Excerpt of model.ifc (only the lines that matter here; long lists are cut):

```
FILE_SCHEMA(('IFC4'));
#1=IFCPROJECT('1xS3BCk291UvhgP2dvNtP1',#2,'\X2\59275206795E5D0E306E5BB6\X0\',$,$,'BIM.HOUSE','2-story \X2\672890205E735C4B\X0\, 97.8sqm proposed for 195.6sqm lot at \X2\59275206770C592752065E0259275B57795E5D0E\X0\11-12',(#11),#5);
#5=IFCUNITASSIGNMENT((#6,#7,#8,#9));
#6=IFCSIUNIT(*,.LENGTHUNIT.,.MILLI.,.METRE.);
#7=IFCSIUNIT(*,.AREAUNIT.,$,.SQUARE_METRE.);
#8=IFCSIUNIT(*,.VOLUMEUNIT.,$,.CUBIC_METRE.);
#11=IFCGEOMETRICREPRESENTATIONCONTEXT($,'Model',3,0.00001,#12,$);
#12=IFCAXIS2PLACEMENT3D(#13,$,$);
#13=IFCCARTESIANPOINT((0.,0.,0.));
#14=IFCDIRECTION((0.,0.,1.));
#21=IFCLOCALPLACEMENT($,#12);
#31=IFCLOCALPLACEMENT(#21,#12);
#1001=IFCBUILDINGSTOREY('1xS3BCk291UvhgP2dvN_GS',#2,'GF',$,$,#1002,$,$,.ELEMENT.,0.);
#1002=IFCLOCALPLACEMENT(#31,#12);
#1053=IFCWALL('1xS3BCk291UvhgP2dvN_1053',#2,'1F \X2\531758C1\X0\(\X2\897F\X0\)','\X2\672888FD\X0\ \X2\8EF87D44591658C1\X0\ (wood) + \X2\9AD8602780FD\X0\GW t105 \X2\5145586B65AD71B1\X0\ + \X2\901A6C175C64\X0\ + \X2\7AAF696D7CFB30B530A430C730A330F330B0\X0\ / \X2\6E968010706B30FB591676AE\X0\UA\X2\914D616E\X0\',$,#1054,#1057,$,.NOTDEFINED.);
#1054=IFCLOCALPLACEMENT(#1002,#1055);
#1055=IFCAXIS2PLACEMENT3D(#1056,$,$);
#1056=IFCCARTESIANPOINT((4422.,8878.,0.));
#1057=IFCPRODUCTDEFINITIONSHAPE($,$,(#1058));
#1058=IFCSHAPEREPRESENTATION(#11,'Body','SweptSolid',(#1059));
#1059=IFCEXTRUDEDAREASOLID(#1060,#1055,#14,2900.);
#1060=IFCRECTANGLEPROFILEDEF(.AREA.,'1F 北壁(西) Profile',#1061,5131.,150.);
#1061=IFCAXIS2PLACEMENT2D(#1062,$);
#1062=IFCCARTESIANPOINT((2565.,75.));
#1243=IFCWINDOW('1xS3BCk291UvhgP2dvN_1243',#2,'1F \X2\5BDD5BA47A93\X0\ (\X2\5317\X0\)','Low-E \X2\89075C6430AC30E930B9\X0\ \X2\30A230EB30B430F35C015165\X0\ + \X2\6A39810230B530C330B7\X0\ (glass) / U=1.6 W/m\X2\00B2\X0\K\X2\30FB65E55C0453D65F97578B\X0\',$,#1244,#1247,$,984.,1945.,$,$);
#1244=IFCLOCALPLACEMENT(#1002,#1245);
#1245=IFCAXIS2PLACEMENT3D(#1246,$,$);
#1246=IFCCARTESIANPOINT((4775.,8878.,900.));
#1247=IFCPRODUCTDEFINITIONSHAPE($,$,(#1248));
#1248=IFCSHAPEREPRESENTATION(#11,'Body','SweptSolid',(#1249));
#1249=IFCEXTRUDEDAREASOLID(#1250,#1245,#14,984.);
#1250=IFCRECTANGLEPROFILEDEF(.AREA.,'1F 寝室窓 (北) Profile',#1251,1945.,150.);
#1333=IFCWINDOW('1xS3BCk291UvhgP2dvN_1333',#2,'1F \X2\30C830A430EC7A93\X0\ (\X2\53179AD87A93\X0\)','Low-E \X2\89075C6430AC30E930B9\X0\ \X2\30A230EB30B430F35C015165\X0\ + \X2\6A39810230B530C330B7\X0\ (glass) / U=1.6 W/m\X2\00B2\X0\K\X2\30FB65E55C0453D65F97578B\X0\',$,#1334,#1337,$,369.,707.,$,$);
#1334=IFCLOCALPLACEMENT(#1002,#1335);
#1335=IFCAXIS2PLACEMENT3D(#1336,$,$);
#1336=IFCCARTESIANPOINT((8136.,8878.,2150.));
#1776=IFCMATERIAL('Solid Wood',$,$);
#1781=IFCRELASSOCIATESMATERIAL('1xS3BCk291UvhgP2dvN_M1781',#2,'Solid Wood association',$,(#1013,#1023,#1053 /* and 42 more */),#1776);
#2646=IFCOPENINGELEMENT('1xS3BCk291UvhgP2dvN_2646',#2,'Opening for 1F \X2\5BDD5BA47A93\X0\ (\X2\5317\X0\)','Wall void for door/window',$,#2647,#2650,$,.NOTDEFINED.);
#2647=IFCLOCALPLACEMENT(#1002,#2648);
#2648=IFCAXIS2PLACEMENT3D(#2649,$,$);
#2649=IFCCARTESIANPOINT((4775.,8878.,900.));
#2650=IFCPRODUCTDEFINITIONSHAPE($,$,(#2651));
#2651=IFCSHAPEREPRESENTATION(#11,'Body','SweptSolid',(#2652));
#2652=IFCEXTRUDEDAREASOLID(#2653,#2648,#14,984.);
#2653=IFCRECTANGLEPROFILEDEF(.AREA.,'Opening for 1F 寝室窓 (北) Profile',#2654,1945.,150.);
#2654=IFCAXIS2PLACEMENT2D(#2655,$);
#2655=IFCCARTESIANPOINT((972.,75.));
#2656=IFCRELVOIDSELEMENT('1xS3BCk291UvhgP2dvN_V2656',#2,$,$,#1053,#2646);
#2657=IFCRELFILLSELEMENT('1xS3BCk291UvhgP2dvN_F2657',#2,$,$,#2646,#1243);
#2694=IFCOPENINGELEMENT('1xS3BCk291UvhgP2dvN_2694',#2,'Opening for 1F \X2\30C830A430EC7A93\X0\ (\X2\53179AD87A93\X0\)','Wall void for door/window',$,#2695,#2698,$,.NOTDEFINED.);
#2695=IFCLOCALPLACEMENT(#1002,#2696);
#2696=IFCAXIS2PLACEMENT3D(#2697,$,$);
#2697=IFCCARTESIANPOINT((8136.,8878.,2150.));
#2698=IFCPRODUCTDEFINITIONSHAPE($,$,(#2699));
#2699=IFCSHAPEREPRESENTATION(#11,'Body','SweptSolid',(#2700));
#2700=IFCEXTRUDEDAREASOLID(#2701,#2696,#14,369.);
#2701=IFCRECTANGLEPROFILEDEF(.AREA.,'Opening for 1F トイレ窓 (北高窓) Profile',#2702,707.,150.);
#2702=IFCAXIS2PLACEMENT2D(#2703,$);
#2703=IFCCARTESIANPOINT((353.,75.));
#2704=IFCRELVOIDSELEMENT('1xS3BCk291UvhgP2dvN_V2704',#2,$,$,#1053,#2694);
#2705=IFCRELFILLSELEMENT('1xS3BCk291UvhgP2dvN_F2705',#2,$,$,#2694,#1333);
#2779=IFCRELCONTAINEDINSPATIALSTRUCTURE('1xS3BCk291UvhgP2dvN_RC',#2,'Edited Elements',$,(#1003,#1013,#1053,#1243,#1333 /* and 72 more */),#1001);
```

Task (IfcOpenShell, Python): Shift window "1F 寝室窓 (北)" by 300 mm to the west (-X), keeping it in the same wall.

```python
import ifcopenshell
import ifcopenshell.api.geometry
import ifcopenshell.util.placement
import ifcopenshell.util.unit

model = ifcopenshell.open("model.ifc")
unit_scale = ifcopenshell.util.unit.calculate_unit_scale(model)

window = model.by_guid("1xS3BCk291UvhgP2dvN_1243")
opening = window.FillsVoids[0].RelatingOpeningElement
wall = opening.VoidsElements[0].RelatingBuildingElement

wall_matrix = ifcopenshell.util.placement.get_local_placement(wall.ObjectPlacement)
shift = wall_matrix[:3, 0] * -0.3 / unit_scale
before = ifcopenshell.util.placement.get_local_placement(window.ObjectPlacement)[:3, 3].copy()

# The window is not placed relative to its opening, so move both.
for product in (opening, window):
    matrix = ifcopenshell.util.placement.get_local_placement(product.ObjectPlacement)
    matrix[:3, 3] += shift
    ifcopenshell.api.geometry.edit_object_placement(model, product=product, matrix=matrix, is_si=False)

after = ifcopenshell.util.placement.get_local_placement(window.ObjectPlacement)[:3, 3]
print("window moved by", (after - before).round(3) + 0.0)

model.write("model_v2.ifc")
```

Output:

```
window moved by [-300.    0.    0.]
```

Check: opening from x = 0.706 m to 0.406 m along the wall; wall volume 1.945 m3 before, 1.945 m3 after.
